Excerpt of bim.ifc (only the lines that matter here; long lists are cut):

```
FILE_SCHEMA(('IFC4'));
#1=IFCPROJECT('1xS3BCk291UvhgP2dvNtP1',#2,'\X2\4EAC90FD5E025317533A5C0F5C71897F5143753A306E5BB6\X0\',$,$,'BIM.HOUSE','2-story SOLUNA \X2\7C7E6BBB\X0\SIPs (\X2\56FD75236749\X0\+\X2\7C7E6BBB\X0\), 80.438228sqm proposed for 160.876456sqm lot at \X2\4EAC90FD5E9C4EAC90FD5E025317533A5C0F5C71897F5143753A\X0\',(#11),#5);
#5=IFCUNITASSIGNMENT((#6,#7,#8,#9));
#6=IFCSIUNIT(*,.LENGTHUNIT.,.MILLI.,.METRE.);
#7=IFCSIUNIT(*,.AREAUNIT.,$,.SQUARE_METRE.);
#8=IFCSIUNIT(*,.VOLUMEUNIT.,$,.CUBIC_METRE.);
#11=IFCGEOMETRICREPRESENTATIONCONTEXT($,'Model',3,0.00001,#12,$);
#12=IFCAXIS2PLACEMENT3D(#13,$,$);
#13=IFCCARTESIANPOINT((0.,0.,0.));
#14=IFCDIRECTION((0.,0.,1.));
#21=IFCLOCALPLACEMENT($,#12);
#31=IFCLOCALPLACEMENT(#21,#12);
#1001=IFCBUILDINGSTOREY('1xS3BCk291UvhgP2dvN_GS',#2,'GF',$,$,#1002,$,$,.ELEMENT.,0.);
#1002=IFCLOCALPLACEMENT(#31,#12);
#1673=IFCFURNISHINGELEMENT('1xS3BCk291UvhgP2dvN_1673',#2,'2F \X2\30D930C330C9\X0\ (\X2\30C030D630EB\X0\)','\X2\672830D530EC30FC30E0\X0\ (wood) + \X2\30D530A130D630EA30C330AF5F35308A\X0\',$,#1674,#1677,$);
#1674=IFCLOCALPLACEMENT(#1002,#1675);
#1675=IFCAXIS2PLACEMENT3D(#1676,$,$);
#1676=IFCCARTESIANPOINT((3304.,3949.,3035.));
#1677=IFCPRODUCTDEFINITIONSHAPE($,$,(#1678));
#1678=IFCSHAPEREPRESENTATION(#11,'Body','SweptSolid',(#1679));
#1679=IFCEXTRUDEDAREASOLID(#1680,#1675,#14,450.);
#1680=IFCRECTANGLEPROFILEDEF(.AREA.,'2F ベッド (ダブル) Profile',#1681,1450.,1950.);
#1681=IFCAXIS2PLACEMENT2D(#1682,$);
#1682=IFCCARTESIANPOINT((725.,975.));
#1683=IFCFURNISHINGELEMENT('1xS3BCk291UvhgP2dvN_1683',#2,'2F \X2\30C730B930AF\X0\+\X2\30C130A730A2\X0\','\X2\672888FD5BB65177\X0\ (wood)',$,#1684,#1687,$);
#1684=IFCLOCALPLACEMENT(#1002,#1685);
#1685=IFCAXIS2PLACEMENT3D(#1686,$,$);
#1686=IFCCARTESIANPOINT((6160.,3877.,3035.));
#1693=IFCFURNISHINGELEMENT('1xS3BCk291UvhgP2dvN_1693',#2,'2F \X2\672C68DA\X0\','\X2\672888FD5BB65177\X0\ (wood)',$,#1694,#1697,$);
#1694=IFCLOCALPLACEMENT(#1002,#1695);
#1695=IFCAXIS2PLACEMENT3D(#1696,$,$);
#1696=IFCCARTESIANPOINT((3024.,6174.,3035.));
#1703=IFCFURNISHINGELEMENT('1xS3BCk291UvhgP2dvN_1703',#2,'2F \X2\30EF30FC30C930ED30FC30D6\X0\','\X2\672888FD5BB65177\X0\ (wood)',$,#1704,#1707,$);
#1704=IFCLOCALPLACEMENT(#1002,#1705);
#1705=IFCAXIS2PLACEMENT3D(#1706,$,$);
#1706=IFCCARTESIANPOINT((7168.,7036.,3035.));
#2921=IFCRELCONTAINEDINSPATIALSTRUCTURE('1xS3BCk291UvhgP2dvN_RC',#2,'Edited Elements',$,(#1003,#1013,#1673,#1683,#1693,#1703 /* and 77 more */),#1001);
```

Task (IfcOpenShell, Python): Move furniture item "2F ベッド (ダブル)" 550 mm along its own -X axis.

```python
import ifcopenshell
import ifcopenshell.api.geometry
import ifcopenshell.util.placement
import ifcopenshell.util.unit

model = ifcopenshell.open("bim.ifc")
unit_scale = ifcopenshell.util.unit.calculate_unit_scale(model)

item = model.by_id(1673)
matrix = ifcopenshell.util.placement.get_local_placement(item.ObjectPlacement)
matrix[:3, 3] -= matrix[:3, 0] * 0.55 / unit_scale
ifcopenshell.api.geometry.edit_object_placement(model, product=item, matrix=matrix, is_si=False)

print(ifcopenshell.util.placement.get_local_placement(item.ObjectPlacement).round(3) + 0.0)

model.write("bim-out.ifc")
```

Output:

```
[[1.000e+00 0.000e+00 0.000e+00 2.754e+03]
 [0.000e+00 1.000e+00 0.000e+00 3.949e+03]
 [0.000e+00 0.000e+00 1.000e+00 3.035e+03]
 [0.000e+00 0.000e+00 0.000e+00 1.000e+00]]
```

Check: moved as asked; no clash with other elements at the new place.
